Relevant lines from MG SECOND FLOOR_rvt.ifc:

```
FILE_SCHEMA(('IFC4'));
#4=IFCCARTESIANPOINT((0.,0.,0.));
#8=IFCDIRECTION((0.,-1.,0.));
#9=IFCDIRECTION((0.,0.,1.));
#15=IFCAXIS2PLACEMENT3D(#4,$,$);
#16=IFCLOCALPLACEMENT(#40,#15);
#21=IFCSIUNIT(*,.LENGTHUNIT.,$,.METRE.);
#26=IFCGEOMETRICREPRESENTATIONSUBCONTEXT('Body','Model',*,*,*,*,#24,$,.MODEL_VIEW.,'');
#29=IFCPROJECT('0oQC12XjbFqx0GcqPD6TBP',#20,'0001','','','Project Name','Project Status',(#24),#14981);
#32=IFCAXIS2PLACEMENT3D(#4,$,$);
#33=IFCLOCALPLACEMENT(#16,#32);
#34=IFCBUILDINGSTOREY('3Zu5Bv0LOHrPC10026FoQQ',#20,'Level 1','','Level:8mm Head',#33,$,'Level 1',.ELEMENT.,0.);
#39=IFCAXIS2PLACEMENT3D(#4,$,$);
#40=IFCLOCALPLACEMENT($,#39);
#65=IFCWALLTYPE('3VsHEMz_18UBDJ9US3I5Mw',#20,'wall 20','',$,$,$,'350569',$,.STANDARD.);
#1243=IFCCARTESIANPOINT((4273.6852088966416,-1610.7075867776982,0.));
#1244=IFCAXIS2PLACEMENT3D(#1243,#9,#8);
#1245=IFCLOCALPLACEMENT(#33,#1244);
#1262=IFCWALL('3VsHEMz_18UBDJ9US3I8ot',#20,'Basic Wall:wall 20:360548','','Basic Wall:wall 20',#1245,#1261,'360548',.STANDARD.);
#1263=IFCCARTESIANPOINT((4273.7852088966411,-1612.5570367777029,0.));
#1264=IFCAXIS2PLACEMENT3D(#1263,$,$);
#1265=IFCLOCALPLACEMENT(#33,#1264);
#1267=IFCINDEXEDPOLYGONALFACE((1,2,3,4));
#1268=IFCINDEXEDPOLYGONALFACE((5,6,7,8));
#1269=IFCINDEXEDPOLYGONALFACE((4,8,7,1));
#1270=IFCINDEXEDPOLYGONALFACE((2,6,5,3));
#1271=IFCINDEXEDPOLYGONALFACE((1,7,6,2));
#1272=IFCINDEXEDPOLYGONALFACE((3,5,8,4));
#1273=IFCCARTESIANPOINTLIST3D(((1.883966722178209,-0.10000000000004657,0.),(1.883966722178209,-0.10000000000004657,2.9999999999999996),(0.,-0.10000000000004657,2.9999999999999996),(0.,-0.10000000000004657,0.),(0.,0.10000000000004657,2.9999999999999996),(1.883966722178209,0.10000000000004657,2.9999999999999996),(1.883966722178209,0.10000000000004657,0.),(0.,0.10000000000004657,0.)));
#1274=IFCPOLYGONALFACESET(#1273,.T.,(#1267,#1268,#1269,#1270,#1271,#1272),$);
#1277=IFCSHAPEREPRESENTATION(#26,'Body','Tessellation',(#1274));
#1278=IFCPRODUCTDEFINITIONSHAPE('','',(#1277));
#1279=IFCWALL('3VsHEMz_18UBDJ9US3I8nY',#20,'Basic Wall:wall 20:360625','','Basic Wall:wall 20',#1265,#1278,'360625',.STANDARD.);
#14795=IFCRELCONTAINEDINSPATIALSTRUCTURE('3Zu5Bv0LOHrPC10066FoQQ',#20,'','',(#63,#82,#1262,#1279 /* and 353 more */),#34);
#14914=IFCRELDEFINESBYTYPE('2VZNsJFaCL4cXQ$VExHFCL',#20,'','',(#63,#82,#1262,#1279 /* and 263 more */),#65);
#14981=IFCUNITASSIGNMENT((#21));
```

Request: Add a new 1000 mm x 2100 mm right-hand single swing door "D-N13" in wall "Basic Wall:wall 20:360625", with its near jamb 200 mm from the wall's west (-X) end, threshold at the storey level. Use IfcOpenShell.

```python
import numpy as np
import ifcopenshell
import ifcopenshell.api.feature
import ifcopenshell.api.geometry
import ifcopenshell.api.root
import ifcopenshell.api.spatial
import ifcopenshell.geom
import ifcopenshell.util.element
import ifcopenshell.util.placement
import ifcopenshell.util.representation
import ifcopenshell.util.shape
import ifcopenshell.util.unit

model = ifcopenshell.open("MG SECOND FLOOR_rvt.ifc")
unit_scale = ifcopenshell.util.unit.calculate_unit_scale(model)
settings = ifcopenshell.geom.settings()


def volume(element):
    """Net volume in cubic metres, openings subtracted."""
    shape = ifcopenshell.geom.create_shape(settings, element)
    return ifcopenshell.util.shape.get_volume(shape.geometry)


wall = model.by_guid("3VsHEMz_18UBDJ9US3I8nY")
storey = ifcopenshell.util.element.get_container(wall, ifc_class="IfcBuildingStorey")
context = ifcopenshell.util.representation.get_context(model, "Model", "Body", "MODEL_VIEW")
before = volume(wall)

width, height, from_end, sill = 1, 2.1, 0.2, 0.0  # metres

# The wall runs along its own X axis, and the end named is its -X end.
wall_shape = ifcopenshell.geom.create_shape(settings, wall)
x, y, z = ifcopenshell.util.shape.get_vertices(wall_shape.geometry).T
start = x.min() + from_end
face, thickness = float(y.min()), float(y.max() - y.min())
wall_matrix = ifcopenshell.util.placement.get_local_placement(wall.ObjectPlacement)
level = ifcopenshell.util.placement.get_local_placement(storey.ObjectPlacement)[2, 3]


def in_wall(x, y):
    """Placement at x, y metres in the wall's axes, at sill height."""
    matrix = wall_matrix.copy()
    matrix[:, 3] = wall_matrix @ np.array([x / unit_scale, y / unit_scale, 0.0, 1.0])
    matrix[2, 3] = level + sill / unit_scale
    return matrix


# Opening: a box that overshoots both wall faces by 50 mm.
opening = ifcopenshell.api.root.create_entity(model, ifc_class="IfcOpeningElement", predefined_type="OPENING")
box = ifcopenshell.api.geometry.add_wall_representation(
    model, context=context, length=width, height=height, thickness=thickness + 0.1
)
ifcopenshell.api.geometry.assign_representation(model, product=opening, representation=box)
ifcopenshell.api.geometry.edit_object_placement(model, product=opening, matrix=in_wall(start, face - 0.05), is_si=False)
ifcopenshell.api.feature.add_feature(model, feature=opening, element=wall)

door = ifcopenshell.api.root.create_entity(model, ifc_class="IfcDoor", name="D-N13", predefined_type="DOOR")
door.OverallWidth, door.OverallHeight = width / unit_scale, height / unit_scale
door.OperationType = "SINGLE_SWING_RIGHT"
body = ifcopenshell.api.geometry.add_door_representation(
    model,
    context=context,
    overall_width=door.OverallWidth,
    overall_height=door.OverallHeight,
    operation_type="SINGLE_SWING_RIGHT",
    lining_properties={"LiningDepth": thickness / unit_scale, "ThresholdDepth": thickness / unit_scale},
)
ifcopenshell.api.geometry.assign_representation(model, product=door, representation=body)
ifcopenshell.api.spatial.assign_container(model, products=[door], relating_structure=storey)
ifcopenshell.api.feature.add_filling(model, opening=opening, element=door)

# The lining spans the wall, so the door starts at the wall face.
ifcopenshell.api.geometry.edit_object_placement(model, product=door, matrix=in_wall(start, face), is_si=False)

after = volume(wall)

print(f"wall volume {before:.3f} -> {after:.3f} m3")

model.write("MG SECOND FLOOR_rvt-out.ifc")
```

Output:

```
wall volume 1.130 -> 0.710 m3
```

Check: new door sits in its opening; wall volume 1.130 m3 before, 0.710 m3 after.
